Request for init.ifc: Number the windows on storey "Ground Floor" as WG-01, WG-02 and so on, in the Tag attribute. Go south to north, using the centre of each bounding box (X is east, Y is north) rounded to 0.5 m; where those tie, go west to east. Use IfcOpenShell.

First a look at what the model holds.

```python
import ifcopenshell
import ifcopenshell.util.element
import ifcopenshell.util.placement

model = ifcopenshell.open("init.ifc")
print(model.schema)
storey = next(s for s in model.by_type("IfcBuildingStorey") if s.Name == "Ground Floor")
windows = [e for e in ifcopenshell.util.element.get_decomposition(storey) if e.is_a("IfcWindow")]
for e in sorted(windows, key=lambda e: e.id()):
    origin = ifcopenshell.util.placement.get_local_placement(e.ObjectPlacement)[:3, 3]
    print(e.id(), e.Tag, e.Name, origin.round(2) + 0.0, sep=" | ")
```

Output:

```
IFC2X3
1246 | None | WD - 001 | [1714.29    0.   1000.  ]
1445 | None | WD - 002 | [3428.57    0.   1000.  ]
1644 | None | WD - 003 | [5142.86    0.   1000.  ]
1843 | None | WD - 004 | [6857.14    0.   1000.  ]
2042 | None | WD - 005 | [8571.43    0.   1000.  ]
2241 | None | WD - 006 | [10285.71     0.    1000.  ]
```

```python
import ifcopenshell
import ifcopenshell.geom
import ifcopenshell.util.element
import ifcopenshell.util.shape

model = ifcopenshell.open("init.ifc")
settings = ifcopenshell.geom.settings()
settings.set("use-world-coords", True)


def centre(element):
    shape = ifcopenshell.geom.create_shape(settings, element)
    return ifcopenshell.util.shape.get_bbox_centroid(shape.geometry)


storey = next(s for s in model.by_type("IfcBuildingStorey") if s.Name == "Ground Floor")
windows = [e for e in ifcopenshell.util.element.get_decomposition(storey) if e.is_a("IfcWindow")]

# Insertion points can sit at a corner or the storey origin, so sort by the geometry (in metres).
centres = {e: centre(e) for e in windows}
windows.sort(key=lambda e: (round(centres[e][1] / 0.5), centres[e][0]))

for i, e in enumerate(windows, start=1):
    number = f"WG-{i:02d}"
    e.Tag = number
    print(e.id(), number)

model.write("init_v2.ifc")
```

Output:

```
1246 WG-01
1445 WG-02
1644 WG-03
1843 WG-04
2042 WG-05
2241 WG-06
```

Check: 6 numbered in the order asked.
